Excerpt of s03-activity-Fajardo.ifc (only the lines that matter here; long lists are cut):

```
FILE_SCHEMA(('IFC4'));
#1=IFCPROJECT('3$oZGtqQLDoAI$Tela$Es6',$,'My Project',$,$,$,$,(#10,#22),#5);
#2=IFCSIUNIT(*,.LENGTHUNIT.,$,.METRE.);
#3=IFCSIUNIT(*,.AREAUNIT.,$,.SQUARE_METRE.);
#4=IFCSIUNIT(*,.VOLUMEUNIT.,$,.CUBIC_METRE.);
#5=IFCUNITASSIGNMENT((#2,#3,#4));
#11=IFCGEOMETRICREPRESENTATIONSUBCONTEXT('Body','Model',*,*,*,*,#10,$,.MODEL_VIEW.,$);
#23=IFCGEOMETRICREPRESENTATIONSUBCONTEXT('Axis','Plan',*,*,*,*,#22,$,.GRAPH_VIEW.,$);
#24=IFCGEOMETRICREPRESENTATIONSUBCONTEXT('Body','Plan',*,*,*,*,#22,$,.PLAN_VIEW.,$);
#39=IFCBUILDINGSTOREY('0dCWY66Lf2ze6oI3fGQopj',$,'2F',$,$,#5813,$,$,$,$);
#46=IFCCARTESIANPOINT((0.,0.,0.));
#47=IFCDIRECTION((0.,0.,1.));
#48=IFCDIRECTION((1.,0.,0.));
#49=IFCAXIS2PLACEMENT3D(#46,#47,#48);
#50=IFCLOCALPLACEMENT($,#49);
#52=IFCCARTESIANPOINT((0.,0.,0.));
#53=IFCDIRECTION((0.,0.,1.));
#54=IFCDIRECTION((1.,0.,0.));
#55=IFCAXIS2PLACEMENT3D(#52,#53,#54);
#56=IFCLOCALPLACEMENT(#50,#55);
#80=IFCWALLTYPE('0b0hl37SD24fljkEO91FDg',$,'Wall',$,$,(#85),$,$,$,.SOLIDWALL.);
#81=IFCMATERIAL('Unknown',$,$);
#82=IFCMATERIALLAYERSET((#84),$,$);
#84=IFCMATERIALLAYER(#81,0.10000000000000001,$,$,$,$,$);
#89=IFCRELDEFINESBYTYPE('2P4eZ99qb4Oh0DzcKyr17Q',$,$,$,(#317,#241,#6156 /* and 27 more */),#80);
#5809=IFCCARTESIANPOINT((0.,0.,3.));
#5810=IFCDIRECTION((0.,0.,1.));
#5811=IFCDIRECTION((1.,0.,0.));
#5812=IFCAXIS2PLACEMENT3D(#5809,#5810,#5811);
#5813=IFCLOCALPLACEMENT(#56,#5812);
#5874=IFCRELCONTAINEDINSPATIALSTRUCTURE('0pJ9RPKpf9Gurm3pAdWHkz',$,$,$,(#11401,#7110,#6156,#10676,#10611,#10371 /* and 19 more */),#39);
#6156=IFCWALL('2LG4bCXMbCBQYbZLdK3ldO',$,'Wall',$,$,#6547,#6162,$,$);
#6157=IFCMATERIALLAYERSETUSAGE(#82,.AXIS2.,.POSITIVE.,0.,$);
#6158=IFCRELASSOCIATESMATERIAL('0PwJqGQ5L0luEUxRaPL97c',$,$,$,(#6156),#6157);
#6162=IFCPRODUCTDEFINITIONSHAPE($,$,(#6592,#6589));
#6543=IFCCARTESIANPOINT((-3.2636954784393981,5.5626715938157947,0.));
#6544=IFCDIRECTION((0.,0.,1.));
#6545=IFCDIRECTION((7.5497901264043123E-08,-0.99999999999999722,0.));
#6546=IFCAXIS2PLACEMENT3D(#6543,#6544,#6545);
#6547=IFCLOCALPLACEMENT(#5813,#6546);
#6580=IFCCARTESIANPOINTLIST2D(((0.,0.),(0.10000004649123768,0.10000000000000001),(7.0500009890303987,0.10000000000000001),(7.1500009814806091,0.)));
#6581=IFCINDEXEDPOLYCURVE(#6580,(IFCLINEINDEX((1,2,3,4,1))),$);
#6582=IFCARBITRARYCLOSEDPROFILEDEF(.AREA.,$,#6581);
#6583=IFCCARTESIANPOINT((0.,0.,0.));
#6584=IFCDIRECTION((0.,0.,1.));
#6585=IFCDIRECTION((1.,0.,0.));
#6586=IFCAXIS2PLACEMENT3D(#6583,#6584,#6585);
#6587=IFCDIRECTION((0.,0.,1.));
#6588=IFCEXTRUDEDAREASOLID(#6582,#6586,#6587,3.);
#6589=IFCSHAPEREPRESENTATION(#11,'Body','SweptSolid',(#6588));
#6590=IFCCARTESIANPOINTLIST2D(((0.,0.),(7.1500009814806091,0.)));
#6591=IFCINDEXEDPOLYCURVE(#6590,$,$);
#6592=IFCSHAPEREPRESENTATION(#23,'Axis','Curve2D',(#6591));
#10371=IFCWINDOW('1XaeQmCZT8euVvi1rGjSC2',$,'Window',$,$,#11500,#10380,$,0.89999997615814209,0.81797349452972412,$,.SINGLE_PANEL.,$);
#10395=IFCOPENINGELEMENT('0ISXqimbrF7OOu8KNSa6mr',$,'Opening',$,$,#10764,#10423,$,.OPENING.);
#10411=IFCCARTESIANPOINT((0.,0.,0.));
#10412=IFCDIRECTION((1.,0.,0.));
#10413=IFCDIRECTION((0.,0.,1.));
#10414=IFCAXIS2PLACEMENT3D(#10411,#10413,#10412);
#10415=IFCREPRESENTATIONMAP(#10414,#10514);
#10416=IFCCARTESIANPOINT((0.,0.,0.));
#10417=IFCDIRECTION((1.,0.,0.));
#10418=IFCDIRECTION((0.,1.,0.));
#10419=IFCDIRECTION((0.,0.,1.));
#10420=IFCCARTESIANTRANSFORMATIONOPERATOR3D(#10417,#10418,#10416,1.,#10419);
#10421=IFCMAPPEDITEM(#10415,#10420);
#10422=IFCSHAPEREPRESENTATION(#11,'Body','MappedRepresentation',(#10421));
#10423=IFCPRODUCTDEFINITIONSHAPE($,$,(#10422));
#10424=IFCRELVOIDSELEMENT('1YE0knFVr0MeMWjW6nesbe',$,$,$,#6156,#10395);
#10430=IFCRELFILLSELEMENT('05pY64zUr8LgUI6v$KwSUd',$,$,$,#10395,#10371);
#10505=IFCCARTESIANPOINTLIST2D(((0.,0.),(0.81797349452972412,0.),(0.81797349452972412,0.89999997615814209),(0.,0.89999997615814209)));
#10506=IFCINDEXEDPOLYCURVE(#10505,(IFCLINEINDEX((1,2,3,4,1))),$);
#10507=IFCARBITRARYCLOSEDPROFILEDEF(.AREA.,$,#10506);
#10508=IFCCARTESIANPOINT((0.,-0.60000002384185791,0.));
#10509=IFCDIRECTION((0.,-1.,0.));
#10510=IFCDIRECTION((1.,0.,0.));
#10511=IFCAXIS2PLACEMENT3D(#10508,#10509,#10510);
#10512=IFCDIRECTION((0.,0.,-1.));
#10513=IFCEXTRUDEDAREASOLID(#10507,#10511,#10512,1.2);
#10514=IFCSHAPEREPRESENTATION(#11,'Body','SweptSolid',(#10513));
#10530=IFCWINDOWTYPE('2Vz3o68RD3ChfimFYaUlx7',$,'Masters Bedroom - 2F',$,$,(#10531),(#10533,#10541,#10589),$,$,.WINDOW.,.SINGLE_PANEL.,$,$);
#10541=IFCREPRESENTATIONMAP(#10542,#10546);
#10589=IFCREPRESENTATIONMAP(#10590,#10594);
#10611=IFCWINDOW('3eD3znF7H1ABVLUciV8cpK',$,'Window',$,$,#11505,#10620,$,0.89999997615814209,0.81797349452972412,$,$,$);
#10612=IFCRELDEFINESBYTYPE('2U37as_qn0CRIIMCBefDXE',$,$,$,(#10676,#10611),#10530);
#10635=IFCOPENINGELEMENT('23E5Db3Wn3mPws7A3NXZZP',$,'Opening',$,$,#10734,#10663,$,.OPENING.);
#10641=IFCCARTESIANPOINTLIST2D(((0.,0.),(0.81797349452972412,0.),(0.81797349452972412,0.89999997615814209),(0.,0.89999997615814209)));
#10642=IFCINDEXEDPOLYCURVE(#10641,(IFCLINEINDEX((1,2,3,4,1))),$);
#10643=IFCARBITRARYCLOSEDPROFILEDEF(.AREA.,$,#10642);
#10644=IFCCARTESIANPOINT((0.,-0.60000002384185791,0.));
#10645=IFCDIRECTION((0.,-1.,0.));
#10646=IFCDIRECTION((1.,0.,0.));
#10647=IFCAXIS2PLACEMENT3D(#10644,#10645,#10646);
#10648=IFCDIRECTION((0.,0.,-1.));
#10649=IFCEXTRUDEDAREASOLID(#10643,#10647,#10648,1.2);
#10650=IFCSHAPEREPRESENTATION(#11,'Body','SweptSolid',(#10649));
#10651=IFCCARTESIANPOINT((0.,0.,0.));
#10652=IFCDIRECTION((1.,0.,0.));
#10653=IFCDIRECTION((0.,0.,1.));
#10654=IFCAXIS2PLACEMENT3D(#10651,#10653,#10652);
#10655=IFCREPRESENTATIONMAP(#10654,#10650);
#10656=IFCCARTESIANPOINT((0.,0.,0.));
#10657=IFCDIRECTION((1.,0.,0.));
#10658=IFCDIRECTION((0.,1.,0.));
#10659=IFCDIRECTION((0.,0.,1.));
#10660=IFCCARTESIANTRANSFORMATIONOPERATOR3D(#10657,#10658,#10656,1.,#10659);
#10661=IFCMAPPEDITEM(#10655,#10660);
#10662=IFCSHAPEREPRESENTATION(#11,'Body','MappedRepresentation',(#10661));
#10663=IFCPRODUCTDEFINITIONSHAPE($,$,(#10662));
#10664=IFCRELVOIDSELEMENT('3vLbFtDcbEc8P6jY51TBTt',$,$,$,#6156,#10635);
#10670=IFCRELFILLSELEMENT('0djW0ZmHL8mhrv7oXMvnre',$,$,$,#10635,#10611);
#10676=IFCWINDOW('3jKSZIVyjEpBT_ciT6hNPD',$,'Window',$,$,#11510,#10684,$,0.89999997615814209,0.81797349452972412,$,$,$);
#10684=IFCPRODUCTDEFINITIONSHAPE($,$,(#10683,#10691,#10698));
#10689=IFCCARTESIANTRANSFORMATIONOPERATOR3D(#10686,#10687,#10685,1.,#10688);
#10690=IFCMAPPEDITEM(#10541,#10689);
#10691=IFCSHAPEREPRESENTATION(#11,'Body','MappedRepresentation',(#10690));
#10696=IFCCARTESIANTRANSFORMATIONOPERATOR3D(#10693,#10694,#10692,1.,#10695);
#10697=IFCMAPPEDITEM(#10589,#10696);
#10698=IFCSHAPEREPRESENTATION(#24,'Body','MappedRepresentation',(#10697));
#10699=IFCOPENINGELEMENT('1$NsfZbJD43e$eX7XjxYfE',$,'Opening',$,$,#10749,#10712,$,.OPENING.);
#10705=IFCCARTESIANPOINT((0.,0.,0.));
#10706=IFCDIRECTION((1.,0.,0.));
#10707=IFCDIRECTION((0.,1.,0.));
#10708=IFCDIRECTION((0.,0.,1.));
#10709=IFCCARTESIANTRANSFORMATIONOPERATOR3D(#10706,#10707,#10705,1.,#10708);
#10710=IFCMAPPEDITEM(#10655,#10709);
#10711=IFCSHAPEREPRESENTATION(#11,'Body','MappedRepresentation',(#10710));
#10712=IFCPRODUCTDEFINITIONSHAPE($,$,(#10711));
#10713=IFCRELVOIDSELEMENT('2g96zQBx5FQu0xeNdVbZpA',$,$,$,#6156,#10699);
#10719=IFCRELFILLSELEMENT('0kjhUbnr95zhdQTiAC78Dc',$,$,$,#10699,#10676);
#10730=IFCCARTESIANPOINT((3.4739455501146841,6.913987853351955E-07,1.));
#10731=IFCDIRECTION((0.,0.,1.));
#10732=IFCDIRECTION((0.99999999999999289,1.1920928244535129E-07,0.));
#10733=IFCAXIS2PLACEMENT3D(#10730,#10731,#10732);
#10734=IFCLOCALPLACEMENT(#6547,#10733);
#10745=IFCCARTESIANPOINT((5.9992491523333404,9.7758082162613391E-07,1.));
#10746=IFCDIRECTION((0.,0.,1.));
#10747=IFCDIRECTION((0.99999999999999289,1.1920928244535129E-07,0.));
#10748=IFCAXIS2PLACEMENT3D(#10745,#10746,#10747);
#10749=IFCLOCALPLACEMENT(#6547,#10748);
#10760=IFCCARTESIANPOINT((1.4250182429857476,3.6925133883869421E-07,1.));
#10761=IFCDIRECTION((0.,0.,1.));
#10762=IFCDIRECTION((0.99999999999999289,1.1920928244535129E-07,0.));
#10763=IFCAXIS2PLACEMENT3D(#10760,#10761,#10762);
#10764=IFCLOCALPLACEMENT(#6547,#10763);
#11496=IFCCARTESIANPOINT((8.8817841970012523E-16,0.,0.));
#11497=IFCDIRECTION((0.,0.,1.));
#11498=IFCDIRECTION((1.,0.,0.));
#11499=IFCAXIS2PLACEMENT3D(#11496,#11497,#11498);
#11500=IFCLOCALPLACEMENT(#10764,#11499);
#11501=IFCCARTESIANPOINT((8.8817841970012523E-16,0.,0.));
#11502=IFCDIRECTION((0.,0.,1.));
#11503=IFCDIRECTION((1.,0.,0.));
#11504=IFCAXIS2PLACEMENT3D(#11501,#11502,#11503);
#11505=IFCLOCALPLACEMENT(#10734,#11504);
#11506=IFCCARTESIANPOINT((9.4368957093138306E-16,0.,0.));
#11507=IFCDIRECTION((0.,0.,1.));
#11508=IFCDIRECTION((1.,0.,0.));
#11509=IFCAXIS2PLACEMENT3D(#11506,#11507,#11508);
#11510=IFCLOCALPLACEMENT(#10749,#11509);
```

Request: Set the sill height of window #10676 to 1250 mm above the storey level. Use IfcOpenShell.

```python
import numpy as np
import ifcopenshell
import ifcopenshell.api.geometry
import ifcopenshell.geom
import ifcopenshell.util.element
import ifcopenshell.util.placement
import ifcopenshell.util.shape
import ifcopenshell.util.unit

model = ifcopenshell.open("s03-activity-Fajardo.ifc")
unit_scale = ifcopenshell.util.unit.calculate_unit_scale(model)

window = model.by_id(10676)
opening = window.FillsVoids[0].RelatingOpeningElement
storey = ifcopenshell.util.element.get_container(window, ifc_class="IfcBuildingStorey")
level = ifcopenshell.util.placement.get_local_placement(storey.ObjectPlacement)[2, 3]

# The opening's origin need not be at the sill, so measure its lowest point.
shape = ifcopenshell.geom.create_shape(ifcopenshell.geom.settings(), opening)
bottom = ifcopenshell.util.shape.get_shape_bottom_elevation(shape, shape.geometry) / unit_scale
dz = level + 1.25 / unit_scale - bottom

shift = np.array([0.0, 0.0, dz])
# The window is placed relative to its opening, so it follows when the opening moves.
matrix = ifcopenshell.util.placement.get_local_placement(opening.ObjectPlacement)
matrix[:3, 3] += shift
ifcopenshell.api.geometry.edit_object_placement(
    model, product=opening, matrix=matrix, is_si=False, should_transform_children=True
)

print(f"moved by {dz * unit_scale:+.3f} m")

model.write("s03-activity-Fajardo-out.ifc")
```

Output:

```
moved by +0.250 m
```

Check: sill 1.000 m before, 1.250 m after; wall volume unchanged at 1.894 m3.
